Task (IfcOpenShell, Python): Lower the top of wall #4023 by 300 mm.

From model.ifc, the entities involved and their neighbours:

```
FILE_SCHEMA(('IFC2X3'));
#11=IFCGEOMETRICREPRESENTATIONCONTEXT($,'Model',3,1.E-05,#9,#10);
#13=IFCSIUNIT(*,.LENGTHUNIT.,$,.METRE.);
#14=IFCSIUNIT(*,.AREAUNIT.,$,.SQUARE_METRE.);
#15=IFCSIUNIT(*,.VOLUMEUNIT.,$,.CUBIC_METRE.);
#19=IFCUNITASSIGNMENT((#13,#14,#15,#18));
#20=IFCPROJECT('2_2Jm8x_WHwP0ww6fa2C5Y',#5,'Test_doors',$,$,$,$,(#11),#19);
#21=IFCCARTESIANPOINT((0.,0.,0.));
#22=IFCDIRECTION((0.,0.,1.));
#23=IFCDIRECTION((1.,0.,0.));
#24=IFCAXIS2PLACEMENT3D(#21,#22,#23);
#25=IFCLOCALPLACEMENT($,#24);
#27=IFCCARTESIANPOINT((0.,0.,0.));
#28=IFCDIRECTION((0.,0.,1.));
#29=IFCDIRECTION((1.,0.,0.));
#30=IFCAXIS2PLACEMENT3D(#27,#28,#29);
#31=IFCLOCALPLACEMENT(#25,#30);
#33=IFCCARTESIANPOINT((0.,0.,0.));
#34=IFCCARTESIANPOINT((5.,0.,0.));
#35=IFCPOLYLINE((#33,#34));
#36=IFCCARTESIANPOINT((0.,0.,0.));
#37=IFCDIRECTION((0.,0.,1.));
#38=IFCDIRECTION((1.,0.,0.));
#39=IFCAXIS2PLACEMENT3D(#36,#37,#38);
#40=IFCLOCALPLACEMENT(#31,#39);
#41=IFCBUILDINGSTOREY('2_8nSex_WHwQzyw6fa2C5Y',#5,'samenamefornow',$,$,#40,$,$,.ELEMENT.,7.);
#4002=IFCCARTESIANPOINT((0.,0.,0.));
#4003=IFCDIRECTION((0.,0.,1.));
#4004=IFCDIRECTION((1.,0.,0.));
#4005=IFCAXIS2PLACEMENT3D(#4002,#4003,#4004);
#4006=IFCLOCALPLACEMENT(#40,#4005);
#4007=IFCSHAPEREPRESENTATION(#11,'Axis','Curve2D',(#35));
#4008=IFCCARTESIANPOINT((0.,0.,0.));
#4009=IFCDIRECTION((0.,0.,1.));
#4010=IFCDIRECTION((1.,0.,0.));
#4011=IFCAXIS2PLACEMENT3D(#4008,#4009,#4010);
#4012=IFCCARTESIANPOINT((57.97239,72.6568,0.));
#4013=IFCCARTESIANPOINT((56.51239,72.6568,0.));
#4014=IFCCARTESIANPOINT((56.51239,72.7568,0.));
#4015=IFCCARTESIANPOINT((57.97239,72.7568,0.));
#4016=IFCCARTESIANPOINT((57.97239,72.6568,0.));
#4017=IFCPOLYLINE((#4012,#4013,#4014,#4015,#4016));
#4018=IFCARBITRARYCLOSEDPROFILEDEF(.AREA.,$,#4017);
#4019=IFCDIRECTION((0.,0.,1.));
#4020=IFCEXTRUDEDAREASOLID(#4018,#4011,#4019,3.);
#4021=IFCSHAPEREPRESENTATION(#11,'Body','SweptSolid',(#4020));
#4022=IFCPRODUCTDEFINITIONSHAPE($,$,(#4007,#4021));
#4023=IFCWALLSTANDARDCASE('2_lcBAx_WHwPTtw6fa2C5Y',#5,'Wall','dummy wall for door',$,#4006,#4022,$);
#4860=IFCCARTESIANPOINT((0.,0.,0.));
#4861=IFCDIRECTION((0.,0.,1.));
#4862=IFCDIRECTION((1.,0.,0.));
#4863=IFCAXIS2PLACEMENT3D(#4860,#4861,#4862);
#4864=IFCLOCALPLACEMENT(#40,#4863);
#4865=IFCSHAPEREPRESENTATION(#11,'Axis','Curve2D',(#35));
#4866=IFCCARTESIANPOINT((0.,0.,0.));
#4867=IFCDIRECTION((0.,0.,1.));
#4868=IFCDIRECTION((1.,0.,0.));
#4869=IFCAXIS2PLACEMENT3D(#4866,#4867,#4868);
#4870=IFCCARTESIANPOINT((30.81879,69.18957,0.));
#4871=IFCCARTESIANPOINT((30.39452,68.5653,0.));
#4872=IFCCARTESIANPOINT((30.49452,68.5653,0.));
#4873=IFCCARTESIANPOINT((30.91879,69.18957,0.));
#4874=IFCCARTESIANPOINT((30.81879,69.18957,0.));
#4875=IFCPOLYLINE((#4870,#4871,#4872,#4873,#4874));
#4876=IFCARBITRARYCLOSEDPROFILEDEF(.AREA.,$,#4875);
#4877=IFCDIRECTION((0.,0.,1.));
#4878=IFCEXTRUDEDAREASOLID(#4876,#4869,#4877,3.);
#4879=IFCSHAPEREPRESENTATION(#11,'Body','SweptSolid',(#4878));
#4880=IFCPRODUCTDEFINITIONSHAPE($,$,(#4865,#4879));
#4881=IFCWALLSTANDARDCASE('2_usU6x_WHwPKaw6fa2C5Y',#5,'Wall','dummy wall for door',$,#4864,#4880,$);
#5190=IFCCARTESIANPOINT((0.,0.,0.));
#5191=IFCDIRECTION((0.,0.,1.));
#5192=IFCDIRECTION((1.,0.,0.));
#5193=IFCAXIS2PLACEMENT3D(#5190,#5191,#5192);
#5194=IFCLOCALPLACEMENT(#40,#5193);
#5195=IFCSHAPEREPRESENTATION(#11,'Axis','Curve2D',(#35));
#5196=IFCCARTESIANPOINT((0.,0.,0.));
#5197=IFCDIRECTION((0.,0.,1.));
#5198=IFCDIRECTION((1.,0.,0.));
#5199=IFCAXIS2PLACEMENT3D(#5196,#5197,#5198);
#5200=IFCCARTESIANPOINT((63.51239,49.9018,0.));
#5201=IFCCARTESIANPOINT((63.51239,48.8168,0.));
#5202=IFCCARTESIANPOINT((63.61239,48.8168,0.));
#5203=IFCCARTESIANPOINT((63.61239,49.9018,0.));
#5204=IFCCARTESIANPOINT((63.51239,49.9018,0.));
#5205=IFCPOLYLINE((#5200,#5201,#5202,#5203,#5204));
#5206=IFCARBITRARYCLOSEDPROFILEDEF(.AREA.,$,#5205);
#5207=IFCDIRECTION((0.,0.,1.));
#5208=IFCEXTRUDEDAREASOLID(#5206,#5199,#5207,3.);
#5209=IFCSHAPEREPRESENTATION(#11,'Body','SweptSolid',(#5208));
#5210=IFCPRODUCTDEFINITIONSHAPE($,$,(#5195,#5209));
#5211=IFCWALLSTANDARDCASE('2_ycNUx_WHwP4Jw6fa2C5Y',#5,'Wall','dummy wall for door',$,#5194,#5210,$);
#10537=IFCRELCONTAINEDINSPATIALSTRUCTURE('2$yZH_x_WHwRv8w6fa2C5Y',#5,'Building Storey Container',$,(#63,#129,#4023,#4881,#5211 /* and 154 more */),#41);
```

```python
import ifcopenshell
import ifcopenshell.geom
import ifcopenshell.util.shape
import ifcopenshell.util.unit

model = ifcopenshell.open("model.ifc")
unit_scale = ifcopenshell.util.unit.calculate_unit_scale(model)
settings = ifcopenshell.geom.settings()


def volume(element):
    """Net volume in cubic metres, openings subtracted."""
    shape = ifcopenshell.geom.create_shape(settings, element)
    return ifcopenshell.util.shape.get_volume(shape.geometry)


wall = model.by_id(4023)
before = volume(wall)

body = next(r for r in wall.Representation.Representations if r.RepresentationIdentifier == "Body")
solid = body.Items[0]
old_height = solid.Depth
solid.Depth -= 0.3 / unit_scale
after = volume(wall)

print(f"height {old_height:g} -> {solid.Depth:g}, volume {before:.3f} -> {after:.3f} m3")

model.write("model-out.ifc")
```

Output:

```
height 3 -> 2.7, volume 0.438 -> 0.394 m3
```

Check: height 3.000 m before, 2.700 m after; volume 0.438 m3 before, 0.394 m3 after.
